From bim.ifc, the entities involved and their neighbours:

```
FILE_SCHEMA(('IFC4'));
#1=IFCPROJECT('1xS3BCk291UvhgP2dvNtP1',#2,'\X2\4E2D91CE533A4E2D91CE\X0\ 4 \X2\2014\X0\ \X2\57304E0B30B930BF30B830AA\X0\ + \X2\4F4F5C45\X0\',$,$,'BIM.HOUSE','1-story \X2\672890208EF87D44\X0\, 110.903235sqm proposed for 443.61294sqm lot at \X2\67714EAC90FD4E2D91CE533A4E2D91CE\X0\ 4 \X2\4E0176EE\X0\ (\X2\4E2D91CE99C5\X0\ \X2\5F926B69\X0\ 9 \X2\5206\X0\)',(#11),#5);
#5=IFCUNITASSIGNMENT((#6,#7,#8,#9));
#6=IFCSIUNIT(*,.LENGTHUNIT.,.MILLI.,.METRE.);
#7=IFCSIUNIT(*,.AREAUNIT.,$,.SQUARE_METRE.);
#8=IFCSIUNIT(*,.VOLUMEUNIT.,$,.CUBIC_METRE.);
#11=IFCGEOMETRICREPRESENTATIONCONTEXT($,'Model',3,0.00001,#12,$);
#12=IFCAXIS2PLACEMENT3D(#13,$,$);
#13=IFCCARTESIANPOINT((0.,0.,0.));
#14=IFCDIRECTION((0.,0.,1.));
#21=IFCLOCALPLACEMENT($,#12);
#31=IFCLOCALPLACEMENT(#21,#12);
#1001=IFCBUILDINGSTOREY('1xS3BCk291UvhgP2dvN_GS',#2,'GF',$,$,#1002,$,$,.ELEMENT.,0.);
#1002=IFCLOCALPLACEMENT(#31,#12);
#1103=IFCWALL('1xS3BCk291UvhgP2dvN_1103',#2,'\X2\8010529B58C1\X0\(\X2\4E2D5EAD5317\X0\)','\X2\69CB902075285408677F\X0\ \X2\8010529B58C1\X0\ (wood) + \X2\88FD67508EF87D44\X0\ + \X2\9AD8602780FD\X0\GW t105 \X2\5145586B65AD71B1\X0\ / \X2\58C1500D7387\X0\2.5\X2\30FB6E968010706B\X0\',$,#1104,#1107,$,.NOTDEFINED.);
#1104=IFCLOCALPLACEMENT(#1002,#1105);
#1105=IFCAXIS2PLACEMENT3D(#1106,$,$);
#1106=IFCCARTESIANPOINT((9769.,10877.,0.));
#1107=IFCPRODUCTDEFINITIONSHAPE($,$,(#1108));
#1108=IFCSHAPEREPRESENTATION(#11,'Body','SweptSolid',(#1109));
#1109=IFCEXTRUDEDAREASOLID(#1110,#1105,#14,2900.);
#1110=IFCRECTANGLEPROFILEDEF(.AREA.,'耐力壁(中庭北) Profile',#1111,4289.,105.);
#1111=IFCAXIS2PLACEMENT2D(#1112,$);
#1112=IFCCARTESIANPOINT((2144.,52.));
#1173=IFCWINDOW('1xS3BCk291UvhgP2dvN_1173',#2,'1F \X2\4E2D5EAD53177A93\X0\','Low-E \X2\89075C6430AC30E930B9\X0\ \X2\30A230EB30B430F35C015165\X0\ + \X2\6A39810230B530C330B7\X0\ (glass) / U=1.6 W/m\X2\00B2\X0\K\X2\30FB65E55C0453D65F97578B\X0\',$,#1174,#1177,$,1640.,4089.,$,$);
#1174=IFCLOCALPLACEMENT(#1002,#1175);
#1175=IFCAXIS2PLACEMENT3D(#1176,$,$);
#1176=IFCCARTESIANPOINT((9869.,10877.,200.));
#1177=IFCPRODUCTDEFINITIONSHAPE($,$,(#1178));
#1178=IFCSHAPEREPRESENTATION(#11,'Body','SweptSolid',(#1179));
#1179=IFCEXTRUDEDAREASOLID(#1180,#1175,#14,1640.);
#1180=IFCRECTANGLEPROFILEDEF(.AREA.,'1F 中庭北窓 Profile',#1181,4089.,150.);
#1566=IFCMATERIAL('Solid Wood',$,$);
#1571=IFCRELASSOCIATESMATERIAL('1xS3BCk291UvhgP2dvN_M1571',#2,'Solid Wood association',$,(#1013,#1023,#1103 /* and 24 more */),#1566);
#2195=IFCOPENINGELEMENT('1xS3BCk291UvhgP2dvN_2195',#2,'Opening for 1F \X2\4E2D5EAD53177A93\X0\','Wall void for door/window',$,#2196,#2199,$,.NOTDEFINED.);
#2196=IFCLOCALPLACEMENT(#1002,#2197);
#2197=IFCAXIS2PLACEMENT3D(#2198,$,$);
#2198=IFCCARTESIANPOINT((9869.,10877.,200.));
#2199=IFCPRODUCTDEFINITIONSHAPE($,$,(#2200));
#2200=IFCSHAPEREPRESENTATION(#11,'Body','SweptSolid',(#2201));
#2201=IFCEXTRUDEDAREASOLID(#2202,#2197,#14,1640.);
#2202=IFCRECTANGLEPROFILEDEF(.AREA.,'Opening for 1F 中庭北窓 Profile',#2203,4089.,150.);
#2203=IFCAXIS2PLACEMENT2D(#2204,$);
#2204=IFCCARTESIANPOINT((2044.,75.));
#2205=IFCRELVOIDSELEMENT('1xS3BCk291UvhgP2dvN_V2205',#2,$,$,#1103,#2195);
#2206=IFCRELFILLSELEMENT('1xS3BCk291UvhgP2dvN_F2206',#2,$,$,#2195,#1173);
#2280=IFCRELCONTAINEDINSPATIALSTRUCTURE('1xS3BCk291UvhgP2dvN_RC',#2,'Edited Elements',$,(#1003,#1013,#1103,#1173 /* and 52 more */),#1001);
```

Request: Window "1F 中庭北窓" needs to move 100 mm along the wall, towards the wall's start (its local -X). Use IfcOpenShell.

```python
import ifcopenshell
import ifcopenshell.api.geometry
import ifcopenshell.util.placement

model = ifcopenshell.open("bim.ifc")

window = model.by_guid("1xS3BCk291UvhgP2dvN_1173")
opening = window.FillsVoids[0].RelatingOpeningElement
wall = opening.VoidsElements[0].RelatingBuildingElement

wall_matrix = ifcopenshell.util.placement.get_local_placement(wall.ObjectPlacement)
shift = wall_matrix[:3, 0] * -100.0
before = ifcopenshell.util.placement.get_local_placement(window.ObjectPlacement)[:3, 3].copy()

# The window is not placed relative to its opening, so move both.
for product in (opening, window):
    matrix = ifcopenshell.util.placement.get_local_placement(product.ObjectPlacement)
    matrix[:3, 3] += shift
    ifcopenshell.api.geometry.edit_object_placement(model, product=product, matrix=matrix, is_si=False)

after = ifcopenshell.util.placement.get_local_placement(window.ObjectPlacement)[:3, 3]
print("window moved by", (after - before).round(3) + 0.0)

model.write("bim_updated.ifc")
```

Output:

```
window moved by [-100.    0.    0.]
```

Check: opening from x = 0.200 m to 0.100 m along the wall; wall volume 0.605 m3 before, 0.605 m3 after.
